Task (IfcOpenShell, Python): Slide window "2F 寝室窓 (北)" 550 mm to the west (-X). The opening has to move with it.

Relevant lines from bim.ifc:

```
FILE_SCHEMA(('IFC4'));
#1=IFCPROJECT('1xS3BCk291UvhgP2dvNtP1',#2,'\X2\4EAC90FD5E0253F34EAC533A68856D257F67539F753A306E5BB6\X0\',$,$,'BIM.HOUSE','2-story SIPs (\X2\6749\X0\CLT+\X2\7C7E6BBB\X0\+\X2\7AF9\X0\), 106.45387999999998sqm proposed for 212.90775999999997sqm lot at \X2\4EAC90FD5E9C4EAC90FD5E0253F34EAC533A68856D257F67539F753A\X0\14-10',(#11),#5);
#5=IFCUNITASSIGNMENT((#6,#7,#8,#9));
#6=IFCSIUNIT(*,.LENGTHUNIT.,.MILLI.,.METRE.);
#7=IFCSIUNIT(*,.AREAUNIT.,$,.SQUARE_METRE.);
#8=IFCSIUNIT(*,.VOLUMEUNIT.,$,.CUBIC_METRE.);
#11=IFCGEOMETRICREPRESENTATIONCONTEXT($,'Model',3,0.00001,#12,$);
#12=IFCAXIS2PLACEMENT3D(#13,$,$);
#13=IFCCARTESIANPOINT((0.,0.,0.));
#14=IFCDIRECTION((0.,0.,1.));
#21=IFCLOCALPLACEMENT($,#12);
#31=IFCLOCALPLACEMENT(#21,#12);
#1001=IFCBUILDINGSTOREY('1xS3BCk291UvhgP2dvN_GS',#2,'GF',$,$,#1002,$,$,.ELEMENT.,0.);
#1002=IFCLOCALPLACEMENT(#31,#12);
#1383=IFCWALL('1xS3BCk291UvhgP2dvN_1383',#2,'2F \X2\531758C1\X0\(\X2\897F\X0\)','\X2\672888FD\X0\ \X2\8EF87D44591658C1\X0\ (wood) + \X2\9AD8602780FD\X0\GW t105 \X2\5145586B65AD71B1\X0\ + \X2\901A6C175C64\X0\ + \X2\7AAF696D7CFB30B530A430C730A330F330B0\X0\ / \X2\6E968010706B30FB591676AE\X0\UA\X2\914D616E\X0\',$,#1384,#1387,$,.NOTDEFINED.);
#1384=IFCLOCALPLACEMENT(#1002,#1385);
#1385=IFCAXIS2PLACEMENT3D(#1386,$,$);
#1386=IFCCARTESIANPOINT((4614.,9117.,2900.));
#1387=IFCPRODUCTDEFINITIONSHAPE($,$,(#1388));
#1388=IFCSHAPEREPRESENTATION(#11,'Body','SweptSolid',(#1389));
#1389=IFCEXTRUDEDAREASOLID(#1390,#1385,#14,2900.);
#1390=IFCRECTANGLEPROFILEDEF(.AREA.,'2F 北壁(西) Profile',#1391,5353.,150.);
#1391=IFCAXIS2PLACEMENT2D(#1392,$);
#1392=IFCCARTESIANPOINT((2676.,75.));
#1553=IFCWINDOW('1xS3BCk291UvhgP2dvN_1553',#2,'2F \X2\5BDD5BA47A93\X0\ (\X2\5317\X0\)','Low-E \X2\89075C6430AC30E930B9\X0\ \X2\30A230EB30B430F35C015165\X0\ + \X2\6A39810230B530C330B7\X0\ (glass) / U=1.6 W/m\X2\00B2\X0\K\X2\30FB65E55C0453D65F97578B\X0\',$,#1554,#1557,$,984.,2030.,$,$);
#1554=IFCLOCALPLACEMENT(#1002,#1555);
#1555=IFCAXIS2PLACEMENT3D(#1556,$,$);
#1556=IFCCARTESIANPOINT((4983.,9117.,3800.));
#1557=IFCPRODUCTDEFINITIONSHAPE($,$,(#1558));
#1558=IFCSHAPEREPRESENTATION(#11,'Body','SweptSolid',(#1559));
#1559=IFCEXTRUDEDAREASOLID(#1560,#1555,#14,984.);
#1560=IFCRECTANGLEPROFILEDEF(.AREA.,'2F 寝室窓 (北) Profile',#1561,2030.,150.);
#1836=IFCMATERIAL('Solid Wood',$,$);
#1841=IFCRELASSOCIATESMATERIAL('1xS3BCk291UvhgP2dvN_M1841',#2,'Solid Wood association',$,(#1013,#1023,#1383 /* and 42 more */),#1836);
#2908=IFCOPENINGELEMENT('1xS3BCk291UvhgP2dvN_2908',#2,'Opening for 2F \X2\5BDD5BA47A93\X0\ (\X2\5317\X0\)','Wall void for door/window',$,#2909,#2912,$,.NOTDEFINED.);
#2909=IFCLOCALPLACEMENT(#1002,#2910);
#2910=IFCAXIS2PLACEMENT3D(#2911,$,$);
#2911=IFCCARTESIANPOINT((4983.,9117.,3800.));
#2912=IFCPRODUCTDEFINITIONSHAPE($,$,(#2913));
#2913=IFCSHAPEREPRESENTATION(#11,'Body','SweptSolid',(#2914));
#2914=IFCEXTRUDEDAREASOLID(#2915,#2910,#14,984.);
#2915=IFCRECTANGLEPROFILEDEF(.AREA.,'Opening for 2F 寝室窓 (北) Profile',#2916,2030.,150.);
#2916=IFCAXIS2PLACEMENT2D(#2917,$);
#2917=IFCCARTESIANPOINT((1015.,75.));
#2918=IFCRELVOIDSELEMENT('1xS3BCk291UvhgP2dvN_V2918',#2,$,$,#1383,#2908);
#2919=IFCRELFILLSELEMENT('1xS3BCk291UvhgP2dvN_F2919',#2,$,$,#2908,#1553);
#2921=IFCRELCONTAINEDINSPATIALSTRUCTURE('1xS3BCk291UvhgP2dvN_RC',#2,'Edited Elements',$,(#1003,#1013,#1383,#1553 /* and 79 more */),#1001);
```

```python
import ifcopenshell
import ifcopenshell.api.geometry
import ifcopenshell.util.placement
import ifcopenshell.util.unit

model = ifcopenshell.open("bim.ifc")
unit_scale = ifcopenshell.util.unit.calculate_unit_scale(model)

window = model.by_id(1553)
opening = window.FillsVoids[0].RelatingOpeningElement
wall = opening.VoidsElements[0].RelatingBuildingElement

wall_matrix = ifcopenshell.util.placement.get_local_placement(wall.ObjectPlacement)
shift = wall_matrix[:3, 0] * -0.55 / unit_scale
before = ifcopenshell.util.placement.get_local_placement(window.ObjectPlacement)[:3, 3].copy()

# The window is not placed relative to its opening, so move both.
for product in (opening, window):
    matrix = ifcopenshell.util.placement.get_local_placement(product.ObjectPlacement)
    matrix[:3, 3] += shift
    ifcopenshell.api.geometry.edit_object_placement(model, product=product, matrix=matrix, is_si=False)

after = ifcopenshell.util.placement.get_local_placement(window.ObjectPlacement)[:3, 3]
print("window moved by", (after - before).round(3) + 0.0)

model.write("bim-out.ifc")
```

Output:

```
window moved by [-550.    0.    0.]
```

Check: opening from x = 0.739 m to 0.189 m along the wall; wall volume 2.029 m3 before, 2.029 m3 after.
